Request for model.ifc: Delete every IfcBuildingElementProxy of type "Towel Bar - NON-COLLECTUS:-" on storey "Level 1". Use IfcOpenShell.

First a look at what the model holds.

```python
import ifcopenshell
import ifcopenshell.util.element

model = ifcopenshell.open("model.ifc")
print(model.schema)
storey = next(s for s in model.by_type("IfcBuildingStorey") if s.Name == "Level 1")
proxies = [e for e in ifcopenshell.util.element.get_decomposition(storey) if e.is_a("IfcBuildingElementProxy")]
seen = {}
for e in proxies:
    element_type = ifcopenshell.util.element.get_type(e)
    name = element_type.Name if element_type not in (None, e) else None
    seen[name] = seen.get(name, 0) + 1
for name, count in sorted(seen.items(), key=str):
    print(count, "x", name)
```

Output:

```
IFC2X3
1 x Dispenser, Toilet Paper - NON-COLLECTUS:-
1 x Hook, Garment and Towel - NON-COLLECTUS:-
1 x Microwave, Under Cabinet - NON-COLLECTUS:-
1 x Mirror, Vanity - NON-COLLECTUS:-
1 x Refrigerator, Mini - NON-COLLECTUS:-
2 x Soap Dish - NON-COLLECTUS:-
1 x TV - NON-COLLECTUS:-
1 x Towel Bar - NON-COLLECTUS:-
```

```python
import ifcopenshell
import ifcopenshell.api.root
import ifcopenshell.util.element

model = ifcopenshell.open("model.ifc")

storey = next(s for s in model.by_type("IfcBuildingStorey") if s.Name == "Level 1")
proxies = [e for e in ifcopenshell.util.element.get_decomposition(storey) if e.is_a("IfcBuildingElementProxy")]
targets = [e for e in proxies if (t := ifcopenshell.util.element.get_type(e)) not in (None, e) and t.Name == "Towel Bar - NON-COLLECTUS:-"]

for e in targets:
    ifcopenshell.api.root.remove_product(model, product=e)
print(len(targets), "removed")

model.write("model_updated.ifc")
```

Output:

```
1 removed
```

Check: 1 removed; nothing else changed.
